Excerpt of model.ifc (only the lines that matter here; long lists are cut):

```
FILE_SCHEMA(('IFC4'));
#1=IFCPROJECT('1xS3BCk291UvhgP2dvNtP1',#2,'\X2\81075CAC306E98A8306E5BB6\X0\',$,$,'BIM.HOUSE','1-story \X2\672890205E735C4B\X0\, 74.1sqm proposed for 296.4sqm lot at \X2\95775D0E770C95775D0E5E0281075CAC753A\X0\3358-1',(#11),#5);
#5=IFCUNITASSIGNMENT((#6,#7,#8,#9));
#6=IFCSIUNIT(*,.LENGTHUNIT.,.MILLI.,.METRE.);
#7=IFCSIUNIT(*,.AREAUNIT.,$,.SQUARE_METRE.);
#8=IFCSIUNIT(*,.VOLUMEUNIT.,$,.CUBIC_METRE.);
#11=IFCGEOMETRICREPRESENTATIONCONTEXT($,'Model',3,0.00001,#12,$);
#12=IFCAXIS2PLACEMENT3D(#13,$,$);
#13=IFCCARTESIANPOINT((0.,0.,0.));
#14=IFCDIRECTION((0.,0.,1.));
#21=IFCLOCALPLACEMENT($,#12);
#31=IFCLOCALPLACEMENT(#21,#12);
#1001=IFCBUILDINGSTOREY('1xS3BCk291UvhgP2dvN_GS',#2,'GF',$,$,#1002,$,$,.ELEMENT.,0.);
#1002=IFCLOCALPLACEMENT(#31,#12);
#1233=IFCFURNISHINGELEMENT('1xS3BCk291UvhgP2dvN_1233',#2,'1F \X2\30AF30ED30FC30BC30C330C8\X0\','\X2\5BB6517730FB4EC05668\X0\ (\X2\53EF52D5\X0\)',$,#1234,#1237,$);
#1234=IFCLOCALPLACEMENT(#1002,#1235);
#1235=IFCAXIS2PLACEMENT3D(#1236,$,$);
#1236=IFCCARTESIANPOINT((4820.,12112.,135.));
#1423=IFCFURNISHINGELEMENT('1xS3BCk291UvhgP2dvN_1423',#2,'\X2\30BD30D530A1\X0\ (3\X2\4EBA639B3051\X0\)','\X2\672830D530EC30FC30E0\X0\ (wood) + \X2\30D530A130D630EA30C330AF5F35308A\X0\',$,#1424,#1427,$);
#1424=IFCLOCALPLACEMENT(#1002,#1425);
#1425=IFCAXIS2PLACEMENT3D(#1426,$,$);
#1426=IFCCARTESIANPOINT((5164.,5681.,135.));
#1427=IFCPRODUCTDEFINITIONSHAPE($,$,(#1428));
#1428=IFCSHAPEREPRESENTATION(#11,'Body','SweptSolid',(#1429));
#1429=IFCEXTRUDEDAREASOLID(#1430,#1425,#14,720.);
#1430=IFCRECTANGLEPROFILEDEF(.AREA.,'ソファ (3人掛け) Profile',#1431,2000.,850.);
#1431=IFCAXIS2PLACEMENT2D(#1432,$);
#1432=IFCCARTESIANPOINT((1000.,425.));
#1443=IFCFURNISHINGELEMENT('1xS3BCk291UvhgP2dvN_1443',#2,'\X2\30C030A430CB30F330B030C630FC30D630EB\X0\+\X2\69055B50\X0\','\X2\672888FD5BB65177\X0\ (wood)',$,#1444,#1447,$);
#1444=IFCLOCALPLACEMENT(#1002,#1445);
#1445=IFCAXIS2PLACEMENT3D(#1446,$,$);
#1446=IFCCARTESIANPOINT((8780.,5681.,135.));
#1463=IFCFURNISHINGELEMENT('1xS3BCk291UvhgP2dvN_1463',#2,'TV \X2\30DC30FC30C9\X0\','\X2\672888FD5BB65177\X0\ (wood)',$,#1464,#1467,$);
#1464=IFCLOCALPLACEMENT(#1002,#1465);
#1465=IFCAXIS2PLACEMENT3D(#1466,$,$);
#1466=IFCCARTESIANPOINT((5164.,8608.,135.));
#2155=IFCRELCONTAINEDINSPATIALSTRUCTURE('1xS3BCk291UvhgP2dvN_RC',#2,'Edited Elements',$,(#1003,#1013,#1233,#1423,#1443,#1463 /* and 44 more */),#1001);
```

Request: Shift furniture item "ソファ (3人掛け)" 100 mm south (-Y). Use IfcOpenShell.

```python
import ifcopenshell
import ifcopenshell.api.geometry
import ifcopenshell.util.placement

model = ifcopenshell.open("model.ifc")

item = model.by_id(1423)
matrix = ifcopenshell.util.placement.get_local_placement(item.ObjectPlacement)
matrix[1, 3] -= 100.0
ifcopenshell.api.geometry.edit_object_placement(model, product=item, matrix=matrix, is_si=False)

print(ifcopenshell.util.placement.get_local_placement(item.ObjectPlacement).round(3) + 0.0)

model.write("model_v2.ifc")
```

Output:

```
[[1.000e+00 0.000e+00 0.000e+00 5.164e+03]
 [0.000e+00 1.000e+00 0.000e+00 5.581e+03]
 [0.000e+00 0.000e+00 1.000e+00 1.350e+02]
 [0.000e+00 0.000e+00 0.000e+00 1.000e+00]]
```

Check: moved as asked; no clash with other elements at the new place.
